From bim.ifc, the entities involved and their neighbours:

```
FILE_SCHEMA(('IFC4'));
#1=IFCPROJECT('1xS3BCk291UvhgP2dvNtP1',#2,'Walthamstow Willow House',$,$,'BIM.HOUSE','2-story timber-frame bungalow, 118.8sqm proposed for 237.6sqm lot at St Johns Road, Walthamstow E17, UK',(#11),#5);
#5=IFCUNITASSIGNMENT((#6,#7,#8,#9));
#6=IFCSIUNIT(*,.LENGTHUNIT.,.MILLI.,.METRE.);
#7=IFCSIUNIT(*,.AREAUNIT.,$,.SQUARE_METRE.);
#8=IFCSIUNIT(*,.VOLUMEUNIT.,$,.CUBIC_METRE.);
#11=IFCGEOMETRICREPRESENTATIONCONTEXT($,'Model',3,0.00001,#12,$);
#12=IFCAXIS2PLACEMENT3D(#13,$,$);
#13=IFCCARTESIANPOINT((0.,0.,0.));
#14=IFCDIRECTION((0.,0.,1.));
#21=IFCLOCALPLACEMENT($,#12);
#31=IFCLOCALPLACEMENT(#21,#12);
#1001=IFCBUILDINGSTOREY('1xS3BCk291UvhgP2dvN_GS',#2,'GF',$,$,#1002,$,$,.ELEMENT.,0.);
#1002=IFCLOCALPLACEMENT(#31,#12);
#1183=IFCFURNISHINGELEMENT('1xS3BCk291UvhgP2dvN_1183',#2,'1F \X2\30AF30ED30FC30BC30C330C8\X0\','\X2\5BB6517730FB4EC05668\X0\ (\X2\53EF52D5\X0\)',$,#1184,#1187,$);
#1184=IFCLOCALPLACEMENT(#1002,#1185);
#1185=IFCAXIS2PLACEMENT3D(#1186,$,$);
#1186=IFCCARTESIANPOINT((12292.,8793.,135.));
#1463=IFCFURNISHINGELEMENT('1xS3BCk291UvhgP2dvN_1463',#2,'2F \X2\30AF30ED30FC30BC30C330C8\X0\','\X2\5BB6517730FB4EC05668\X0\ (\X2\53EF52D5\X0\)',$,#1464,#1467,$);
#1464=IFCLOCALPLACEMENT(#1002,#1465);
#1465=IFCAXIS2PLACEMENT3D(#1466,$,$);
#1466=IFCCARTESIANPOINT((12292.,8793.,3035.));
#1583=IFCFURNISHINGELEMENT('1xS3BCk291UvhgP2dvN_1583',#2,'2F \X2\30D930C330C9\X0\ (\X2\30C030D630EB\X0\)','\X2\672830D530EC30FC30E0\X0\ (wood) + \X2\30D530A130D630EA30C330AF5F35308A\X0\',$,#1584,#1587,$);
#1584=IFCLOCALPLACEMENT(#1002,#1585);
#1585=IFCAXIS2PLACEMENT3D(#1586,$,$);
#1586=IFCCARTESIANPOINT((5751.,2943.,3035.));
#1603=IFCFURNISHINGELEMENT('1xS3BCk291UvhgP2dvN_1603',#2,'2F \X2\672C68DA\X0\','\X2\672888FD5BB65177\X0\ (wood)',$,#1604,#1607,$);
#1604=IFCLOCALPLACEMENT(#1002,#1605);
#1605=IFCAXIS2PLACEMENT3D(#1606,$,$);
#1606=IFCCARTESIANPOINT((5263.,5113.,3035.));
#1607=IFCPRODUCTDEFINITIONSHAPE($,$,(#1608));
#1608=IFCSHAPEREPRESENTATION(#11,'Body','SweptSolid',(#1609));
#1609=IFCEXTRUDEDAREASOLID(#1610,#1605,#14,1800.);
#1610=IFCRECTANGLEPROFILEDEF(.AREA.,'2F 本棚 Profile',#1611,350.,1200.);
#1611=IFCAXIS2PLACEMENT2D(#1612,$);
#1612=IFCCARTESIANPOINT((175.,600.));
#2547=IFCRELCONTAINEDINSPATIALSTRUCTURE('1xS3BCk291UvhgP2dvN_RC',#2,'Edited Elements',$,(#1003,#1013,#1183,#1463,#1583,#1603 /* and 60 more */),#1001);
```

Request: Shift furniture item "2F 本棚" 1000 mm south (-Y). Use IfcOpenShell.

```python
import ifcopenshell
import ifcopenshell.api.geometry
import ifcopenshell.util.placement
import ifcopenshell.util.unit

model = ifcopenshell.open("bim.ifc")
unit_scale = ifcopenshell.util.unit.calculate_unit_scale(model)

item = model.by_guid("1xS3BCk291UvhgP2dvN_1603")
matrix = ifcopenshell.util.placement.get_local_placement(item.ObjectPlacement)
matrix[1, 3] -= 1 / unit_scale
ifcopenshell.api.geometry.edit_object_placement(model, product=item, matrix=matrix, is_si=False)

print(ifcopenshell.util.placement.get_local_placement(item.ObjectPlacement).round(3) + 0.0)

model.write("bim_updated.ifc")
```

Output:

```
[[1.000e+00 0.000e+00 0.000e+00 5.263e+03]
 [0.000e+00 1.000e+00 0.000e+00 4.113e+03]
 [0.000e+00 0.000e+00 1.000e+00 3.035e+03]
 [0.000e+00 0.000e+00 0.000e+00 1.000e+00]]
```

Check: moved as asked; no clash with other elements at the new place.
